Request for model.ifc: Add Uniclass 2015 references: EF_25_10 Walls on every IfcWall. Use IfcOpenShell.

First a look at what the model holds.

```python
import ifcopenshell

model = ifcopenshell.open("model.ifc")
print(model.schema)
print("classifications:", [c.Name for c in model.by_type("IfcClassification")])
for ifc_class in ("IfcDoor", "IfcRoof", "IfcStair", "IfcWall", "IfcWindow"):
    print(ifc_class, len(model.by_type(ifc_class)))
```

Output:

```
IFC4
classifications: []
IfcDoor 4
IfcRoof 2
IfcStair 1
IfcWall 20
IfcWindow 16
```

```python
import ifcopenshell
import ifcopenshell.api.classification

model = ifcopenshell.open("model.ifc")

system = ifcopenshell.api.classification.add_classification(model, classification="Uniclass 2015")

codes = {
    "IfcWall": ("EF_25_10", "Walls"),
}
for ifc_class, (code, name) in codes.items():
    products = model.by_type(ifc_class)
    ifcopenshell.api.classification.add_reference(
        model, products=products, classification=system, identification=code, name=name
    )
    print(code, len(products))

model.write("model_updated.ifc")
```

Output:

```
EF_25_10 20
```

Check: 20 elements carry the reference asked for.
